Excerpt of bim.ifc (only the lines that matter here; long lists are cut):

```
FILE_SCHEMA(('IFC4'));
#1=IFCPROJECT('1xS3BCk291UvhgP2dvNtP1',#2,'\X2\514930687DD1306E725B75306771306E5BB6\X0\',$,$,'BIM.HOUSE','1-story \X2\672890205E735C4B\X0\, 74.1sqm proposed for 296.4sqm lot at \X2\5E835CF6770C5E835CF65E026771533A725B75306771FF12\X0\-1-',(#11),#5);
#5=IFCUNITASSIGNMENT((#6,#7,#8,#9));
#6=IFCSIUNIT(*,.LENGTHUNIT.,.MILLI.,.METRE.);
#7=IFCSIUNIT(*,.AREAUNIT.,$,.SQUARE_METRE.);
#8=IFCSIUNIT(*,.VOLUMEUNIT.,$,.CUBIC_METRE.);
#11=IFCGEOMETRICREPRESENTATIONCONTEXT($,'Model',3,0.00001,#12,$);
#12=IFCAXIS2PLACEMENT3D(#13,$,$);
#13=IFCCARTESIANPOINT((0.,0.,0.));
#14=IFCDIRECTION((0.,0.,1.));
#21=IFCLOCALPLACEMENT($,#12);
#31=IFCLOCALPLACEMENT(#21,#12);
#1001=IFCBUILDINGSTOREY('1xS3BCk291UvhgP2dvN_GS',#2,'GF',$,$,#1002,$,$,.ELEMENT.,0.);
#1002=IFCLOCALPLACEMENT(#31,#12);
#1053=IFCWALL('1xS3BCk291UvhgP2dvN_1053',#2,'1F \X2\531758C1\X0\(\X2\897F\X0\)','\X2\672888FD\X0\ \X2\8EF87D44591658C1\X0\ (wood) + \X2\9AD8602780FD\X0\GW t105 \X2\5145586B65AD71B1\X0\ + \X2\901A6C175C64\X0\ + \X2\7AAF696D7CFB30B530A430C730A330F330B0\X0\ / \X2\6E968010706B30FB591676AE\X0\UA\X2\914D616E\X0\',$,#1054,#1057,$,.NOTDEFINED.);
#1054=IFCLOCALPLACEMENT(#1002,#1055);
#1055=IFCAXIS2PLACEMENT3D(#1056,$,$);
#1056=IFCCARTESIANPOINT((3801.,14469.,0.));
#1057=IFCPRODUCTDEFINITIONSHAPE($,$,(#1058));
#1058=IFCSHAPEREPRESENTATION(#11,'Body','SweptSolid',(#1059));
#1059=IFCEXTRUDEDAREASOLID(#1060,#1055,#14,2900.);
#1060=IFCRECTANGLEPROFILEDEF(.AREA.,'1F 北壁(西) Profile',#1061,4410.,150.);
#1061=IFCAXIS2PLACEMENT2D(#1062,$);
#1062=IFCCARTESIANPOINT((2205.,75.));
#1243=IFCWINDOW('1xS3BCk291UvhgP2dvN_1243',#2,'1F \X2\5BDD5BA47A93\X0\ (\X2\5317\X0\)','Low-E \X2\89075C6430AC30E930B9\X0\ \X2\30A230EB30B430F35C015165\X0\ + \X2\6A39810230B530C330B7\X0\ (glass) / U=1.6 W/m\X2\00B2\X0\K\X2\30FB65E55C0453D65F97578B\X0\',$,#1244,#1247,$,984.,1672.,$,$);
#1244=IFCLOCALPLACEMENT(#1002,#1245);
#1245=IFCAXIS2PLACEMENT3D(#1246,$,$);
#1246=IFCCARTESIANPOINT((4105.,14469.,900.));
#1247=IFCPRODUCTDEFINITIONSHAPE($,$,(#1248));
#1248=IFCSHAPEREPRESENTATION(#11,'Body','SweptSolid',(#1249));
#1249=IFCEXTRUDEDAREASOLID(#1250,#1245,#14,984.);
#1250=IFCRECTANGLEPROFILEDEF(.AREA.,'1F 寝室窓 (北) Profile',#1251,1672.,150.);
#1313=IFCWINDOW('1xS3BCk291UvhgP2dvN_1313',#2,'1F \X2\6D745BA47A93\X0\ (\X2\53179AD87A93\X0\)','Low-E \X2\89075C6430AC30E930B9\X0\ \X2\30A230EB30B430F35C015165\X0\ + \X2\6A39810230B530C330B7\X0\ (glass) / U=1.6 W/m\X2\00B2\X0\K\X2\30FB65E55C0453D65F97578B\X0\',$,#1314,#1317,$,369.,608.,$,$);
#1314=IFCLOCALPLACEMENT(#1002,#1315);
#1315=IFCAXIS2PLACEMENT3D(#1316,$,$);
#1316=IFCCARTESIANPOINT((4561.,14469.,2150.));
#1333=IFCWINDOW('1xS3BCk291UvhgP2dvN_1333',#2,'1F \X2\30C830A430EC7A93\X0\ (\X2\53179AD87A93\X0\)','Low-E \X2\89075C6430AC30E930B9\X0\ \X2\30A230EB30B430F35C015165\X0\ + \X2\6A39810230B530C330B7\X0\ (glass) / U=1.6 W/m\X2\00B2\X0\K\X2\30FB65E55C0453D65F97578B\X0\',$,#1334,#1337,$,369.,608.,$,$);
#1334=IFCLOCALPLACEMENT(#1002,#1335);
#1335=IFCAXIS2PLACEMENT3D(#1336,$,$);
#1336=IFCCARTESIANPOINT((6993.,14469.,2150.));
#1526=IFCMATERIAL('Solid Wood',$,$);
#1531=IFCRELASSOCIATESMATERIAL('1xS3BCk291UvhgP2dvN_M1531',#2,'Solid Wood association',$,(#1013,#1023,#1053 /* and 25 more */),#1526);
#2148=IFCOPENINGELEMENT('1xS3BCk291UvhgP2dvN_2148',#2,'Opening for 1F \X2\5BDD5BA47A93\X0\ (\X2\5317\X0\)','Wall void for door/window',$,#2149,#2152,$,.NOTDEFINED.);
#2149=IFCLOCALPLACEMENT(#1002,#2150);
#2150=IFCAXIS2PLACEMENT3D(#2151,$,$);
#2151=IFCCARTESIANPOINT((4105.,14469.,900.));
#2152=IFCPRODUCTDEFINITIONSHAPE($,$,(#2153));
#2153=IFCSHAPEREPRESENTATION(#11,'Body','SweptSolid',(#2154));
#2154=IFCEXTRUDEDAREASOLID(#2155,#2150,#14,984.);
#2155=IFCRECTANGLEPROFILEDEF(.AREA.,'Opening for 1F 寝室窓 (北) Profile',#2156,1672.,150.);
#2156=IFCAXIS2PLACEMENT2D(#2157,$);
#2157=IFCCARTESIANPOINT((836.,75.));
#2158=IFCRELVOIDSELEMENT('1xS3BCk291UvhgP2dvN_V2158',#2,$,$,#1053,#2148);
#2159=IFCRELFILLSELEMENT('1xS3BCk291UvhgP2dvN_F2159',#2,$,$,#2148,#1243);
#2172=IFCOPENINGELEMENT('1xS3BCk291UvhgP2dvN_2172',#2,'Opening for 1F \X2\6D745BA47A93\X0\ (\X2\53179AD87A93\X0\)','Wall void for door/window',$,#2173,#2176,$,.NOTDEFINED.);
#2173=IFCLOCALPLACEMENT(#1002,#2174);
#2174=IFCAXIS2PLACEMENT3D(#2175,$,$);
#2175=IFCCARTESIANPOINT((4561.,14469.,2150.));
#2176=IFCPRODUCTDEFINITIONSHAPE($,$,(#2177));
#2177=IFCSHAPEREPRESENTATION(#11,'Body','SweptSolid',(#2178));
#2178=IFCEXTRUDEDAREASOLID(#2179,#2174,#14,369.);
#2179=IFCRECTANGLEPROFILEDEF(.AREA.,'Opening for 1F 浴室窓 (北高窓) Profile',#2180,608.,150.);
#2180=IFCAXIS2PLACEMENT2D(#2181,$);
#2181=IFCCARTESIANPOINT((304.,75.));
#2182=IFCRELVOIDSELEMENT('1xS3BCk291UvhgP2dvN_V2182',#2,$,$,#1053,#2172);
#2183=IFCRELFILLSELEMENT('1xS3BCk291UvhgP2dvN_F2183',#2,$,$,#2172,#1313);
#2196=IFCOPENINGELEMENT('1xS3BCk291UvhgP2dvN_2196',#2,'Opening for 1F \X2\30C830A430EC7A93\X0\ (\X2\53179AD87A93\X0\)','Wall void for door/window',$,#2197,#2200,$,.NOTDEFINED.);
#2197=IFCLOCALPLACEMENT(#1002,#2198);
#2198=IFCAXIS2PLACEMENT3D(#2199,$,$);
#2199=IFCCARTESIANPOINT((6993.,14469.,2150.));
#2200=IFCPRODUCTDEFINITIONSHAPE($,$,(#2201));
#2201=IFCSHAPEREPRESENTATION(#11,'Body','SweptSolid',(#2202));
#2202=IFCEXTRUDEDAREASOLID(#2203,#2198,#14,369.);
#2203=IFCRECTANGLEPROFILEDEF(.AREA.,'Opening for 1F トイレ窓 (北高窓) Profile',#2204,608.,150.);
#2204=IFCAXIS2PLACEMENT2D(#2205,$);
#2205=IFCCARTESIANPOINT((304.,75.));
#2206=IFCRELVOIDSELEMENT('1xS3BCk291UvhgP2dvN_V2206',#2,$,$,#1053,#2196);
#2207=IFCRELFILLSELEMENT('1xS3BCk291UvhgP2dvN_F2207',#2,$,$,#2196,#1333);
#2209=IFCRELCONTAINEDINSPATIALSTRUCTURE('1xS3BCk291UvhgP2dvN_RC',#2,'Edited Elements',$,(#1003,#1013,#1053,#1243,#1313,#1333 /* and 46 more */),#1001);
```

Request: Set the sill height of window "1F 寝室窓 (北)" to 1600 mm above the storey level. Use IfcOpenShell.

```python
import numpy as np
import ifcopenshell
import ifcopenshell.api.geometry
import ifcopenshell.geom
import ifcopenshell.util.element
import ifcopenshell.util.placement
import ifcopenshell.util.shape
import ifcopenshell.util.unit

model = ifcopenshell.open("bim.ifc")
unit_scale = ifcopenshell.util.unit.calculate_unit_scale(model)

window = model.by_id(1243)
opening = window.FillsVoids[0].RelatingOpeningElement
storey = ifcopenshell.util.element.get_container(window, ifc_class="IfcBuildingStorey")
level = ifcopenshell.util.placement.get_local_placement(storey.ObjectPlacement)[2, 3]

# The opening's origin need not be at the sill, so measure its lowest point.
shape = ifcopenshell.geom.create_shape(ifcopenshell.geom.settings(), opening)
bottom = ifcopenshell.util.shape.get_shape_bottom_elevation(shape, shape.geometry) / unit_scale
dz = level + 1600.0 - bottom

shift = np.array([0.0, 0.0, dz])
# The window is not placed relative to its opening, so move both.
for product in (opening, window):
    matrix = ifcopenshell.util.placement.get_local_placement(product.ObjectPlacement)
    matrix[:3, 3] += shift
    ifcopenshell.api.geometry.edit_object_placement(model, product=product, matrix=matrix, is_si=False)

print(f"moved by {dz * unit_scale:+.3f} m")

model.write("bim_v2.ifc")
```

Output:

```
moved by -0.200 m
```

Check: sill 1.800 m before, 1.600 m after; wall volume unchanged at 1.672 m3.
